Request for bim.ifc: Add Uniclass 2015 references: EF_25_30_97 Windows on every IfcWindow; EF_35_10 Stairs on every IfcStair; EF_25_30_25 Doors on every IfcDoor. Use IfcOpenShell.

First a look at what the model holds.

```python
import ifcopenshell

model = ifcopenshell.open("bim.ifc")
print(model.schema)
print("classifications:", [c.Name for c in model.by_type("IfcClassification")])
for ifc_class in ("IfcDoor", "IfcRoof", "IfcStair", "IfcWall", "IfcWindow"):
    print(ifc_class, len(model.by_type(ifc_class)))
```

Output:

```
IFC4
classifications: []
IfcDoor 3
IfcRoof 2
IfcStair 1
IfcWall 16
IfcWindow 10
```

```python
import ifcopenshell
import ifcopenshell.api.classification

model = ifcopenshell.open("bim.ifc")

system = ifcopenshell.api.classification.add_classification(model, classification="Uniclass 2015")

codes = {
    "IfcWindow": ("EF_25_30_97", "Windows"),
    "IfcStair": ("EF_35_10", "Stairs"),
    "IfcDoor": ("EF_25_30_25", "Doors"),
}
for ifc_class, (code, name) in codes.items():
    products = model.by_type(ifc_class)
    ifcopenshell.api.classification.add_reference(
        model, products=products, classification=system, identification=code, name=name
    )
    print(code, len(products))

model.write("bim-out.ifc")
```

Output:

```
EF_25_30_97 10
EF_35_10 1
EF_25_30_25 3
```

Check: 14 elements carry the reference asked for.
